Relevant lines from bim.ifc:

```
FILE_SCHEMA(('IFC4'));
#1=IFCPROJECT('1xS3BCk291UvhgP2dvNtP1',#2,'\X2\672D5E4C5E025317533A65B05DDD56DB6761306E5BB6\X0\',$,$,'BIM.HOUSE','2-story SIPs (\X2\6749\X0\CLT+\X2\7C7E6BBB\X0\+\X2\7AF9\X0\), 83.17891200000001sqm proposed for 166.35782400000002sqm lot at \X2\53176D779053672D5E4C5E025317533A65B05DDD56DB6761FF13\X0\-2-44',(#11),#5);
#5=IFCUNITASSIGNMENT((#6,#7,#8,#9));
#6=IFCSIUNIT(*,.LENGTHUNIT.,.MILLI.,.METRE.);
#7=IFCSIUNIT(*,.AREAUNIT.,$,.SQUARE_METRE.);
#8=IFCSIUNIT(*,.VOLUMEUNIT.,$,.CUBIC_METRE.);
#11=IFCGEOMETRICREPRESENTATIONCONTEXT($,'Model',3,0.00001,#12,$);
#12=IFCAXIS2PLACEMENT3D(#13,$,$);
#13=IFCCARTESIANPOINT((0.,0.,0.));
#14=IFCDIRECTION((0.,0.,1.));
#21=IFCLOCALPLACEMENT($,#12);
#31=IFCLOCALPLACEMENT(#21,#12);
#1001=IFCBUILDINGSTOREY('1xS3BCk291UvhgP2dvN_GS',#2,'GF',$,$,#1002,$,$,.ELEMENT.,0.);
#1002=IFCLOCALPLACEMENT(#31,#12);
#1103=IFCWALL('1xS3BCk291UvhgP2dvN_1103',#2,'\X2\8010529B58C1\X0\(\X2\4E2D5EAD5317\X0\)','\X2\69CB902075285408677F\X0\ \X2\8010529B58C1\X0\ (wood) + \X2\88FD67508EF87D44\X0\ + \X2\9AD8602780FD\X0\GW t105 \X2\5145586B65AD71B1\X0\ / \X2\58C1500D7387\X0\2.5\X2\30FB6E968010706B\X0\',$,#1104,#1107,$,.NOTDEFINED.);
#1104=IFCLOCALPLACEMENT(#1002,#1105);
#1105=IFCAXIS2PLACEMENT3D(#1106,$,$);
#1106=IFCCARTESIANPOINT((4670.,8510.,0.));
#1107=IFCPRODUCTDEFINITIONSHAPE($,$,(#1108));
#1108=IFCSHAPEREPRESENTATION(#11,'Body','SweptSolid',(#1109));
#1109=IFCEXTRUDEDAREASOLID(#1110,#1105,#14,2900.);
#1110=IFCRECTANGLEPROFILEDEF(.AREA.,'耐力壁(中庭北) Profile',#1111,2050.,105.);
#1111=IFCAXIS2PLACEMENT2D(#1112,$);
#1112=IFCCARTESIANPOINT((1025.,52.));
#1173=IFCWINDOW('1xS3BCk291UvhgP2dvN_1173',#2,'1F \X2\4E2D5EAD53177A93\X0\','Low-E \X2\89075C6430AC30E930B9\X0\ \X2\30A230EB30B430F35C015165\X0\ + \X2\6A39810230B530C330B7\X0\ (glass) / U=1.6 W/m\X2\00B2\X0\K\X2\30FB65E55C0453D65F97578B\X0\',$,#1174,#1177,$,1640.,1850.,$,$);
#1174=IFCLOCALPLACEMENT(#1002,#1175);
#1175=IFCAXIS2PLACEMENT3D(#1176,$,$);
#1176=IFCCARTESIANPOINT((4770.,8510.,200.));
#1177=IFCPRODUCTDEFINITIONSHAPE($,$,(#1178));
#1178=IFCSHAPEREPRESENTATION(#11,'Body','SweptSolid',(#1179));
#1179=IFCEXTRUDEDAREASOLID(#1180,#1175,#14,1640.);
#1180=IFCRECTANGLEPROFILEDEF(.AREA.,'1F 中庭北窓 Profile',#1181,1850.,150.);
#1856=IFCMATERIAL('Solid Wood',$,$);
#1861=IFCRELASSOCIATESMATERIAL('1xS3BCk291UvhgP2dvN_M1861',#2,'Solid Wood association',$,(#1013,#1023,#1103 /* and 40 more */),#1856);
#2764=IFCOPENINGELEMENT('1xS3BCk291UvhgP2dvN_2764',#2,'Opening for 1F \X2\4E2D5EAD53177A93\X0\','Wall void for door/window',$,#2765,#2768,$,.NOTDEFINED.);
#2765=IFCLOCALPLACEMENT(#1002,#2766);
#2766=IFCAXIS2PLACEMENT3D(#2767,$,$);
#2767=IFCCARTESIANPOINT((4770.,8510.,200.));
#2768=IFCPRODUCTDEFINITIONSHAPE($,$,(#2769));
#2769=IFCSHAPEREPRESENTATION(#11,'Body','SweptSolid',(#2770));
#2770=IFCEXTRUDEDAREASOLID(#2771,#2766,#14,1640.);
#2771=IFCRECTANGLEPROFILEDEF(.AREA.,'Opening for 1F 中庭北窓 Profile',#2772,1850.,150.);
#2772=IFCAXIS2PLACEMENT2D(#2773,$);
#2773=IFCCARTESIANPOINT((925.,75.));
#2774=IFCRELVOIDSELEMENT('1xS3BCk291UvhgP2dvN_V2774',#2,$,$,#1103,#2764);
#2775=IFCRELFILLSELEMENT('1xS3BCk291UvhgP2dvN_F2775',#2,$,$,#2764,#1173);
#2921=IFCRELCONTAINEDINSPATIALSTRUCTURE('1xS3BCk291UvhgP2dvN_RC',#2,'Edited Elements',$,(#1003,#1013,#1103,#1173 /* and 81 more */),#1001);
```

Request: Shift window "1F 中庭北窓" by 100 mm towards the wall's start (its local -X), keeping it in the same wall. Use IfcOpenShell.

```python
import ifcopenshell
import ifcopenshell.api.geometry
import ifcopenshell.util.placement
import ifcopenshell.util.unit

model = ifcopenshell.open("bim.ifc")
unit_scale = ifcopenshell.util.unit.calculate_unit_scale(model)

window = model.by_id(1173)
opening = window.FillsVoids[0].RelatingOpeningElement
wall = opening.VoidsElements[0].RelatingBuildingElement

wall_matrix = ifcopenshell.util.placement.get_local_placement(wall.ObjectPlacement)
shift = wall_matrix[:3, 0] * -0.1 / unit_scale
before = ifcopenshell.util.placement.get_local_placement(window.ObjectPlacement)[:3, 3].copy()

# The window is not placed relative to its opening, so move both.
for product in (opening, window):
    matrix = ifcopenshell.util.placement.get_local_placement(product.ObjectPlacement)
    matrix[:3, 3] += shift
    ifcopenshell.api.geometry.edit_object_placement(model, product=product, matrix=matrix, is_si=False)

after = ifcopenshell.util.placement.get_local_placement(window.ObjectPlacement)[:3, 3]
print("window moved by", (after - before).round(3) + 0.0)

model.write("bim-out.ifc")
```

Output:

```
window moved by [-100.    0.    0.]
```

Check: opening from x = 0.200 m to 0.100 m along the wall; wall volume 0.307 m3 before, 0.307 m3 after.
